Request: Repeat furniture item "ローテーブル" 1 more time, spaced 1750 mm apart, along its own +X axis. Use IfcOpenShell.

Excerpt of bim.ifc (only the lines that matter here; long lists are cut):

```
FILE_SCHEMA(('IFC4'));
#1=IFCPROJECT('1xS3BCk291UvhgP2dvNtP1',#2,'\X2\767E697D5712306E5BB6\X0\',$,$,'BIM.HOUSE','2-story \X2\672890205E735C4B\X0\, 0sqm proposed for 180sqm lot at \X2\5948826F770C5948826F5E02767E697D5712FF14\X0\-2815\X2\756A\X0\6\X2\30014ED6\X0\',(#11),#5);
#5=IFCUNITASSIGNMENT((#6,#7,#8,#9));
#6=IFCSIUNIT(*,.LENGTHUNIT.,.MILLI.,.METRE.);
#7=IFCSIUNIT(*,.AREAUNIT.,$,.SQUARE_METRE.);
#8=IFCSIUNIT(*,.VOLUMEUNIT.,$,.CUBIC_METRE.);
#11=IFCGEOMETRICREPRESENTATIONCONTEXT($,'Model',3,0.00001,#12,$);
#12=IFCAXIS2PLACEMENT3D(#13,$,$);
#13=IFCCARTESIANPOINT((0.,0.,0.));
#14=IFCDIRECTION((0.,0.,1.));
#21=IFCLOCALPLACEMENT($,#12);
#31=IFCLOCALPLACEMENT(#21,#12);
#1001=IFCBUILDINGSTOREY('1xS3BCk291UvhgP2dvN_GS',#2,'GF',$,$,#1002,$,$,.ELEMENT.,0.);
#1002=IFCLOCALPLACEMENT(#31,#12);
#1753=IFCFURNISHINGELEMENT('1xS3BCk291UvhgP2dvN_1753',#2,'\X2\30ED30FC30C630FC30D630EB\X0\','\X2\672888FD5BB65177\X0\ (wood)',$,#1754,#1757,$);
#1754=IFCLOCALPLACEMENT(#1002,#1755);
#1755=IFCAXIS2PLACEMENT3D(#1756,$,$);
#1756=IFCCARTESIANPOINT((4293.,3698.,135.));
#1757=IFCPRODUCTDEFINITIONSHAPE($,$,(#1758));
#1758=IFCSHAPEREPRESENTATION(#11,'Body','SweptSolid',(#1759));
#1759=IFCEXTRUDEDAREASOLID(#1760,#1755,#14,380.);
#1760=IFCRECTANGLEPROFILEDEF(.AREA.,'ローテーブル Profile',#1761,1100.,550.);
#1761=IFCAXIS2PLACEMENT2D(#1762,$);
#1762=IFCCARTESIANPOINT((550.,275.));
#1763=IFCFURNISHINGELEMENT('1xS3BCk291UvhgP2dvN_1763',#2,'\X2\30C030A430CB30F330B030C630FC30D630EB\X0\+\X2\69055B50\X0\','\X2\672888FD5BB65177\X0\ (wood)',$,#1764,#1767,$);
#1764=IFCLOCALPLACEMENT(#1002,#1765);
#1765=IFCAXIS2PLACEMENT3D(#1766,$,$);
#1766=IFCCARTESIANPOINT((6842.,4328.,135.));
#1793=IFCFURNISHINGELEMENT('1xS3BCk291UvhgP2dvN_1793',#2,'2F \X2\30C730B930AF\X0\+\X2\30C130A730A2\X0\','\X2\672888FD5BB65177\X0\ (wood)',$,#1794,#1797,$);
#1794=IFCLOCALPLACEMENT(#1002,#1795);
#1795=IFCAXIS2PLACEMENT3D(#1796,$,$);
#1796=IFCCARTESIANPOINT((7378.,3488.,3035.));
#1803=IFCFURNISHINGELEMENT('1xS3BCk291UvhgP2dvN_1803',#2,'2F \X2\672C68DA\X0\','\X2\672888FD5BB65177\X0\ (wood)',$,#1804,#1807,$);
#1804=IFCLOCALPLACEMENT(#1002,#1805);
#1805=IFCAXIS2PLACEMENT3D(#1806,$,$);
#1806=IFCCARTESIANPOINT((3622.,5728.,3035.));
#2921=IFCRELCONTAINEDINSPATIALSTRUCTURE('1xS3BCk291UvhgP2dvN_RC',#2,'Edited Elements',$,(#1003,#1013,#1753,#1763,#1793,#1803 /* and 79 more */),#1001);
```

```python
import ifcopenshell
import ifcopenshell.api.geometry
import ifcopenshell.api.root
import ifcopenshell.util.element
import ifcopenshell.util.placement
import ifcopenshell.util.unit

model = ifcopenshell.open("bim.ifc")
unit_scale = ifcopenshell.util.unit.calculate_unit_scale(model)


def reuse_history(source, copy):
    """copy_class also copies each property set's owner history, people and application; keep the originals."""
    for rel in copy.IsDefinedBy:
        if rel.is_a("IfcRelDefinesByProperties") and (history := rel.RelatingPropertyDefinition.OwnerHistory):
            rel.RelatingPropertyDefinition.OwnerHistory = source.OwnerHistory
            ifcopenshell.util.element.remove_deep2(model, history)


source = model.by_guid("1xS3BCk291UvhgP2dvN_1753")
base = ifcopenshell.util.placement.get_local_placement(source.ObjectPlacement)
step = base[:3, 0] * 1.75 / unit_scale

for i in range(1, 2):
    copy = ifcopenshell.api.root.copy_class(model, product=source)
    copy.Representation = ifcopenshell.util.element.copy_deep(
        model, source.Representation, exclude=["IfcGeometricRepresentationContext", "IfcRepresentationMap"]
    )
    reuse_history(source, copy)
    matrix = base.copy()
    matrix[:3, 3] += i * step
    print("added at", matrix[:3, 3].round(3) + 0.0)
    ifcopenshell.api.geometry.edit_object_placement(model, product=copy, matrix=matrix, is_si=False)

model.write("bim_updated.ifc")
```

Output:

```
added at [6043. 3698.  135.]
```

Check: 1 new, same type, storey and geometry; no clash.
